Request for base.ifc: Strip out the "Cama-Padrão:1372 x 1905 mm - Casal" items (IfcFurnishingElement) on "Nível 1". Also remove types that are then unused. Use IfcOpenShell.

First a look at what the model holds.

```python
import ifcopenshell
import ifcopenshell.util.element

model = ifcopenshell.open("base.ifc")
print(model.schema)
storey = next(s for s in model.by_type("IfcBuildingStorey") if s.Name == "Nível 1")
furniture = [e for e in ifcopenshell.util.element.get_decomposition(storey) if e.is_a("IfcFurnishingElement")]
seen = {}
for e in furniture:
    element_type = ifcopenshell.util.element.get_type(e)
    name = element_type.Name if element_type not in (None, e) else None
    seen[name] = seen.get(name, 0) + 1
for name, count in sorted(seen.items(), key=str):
    print(count, "x", name)
```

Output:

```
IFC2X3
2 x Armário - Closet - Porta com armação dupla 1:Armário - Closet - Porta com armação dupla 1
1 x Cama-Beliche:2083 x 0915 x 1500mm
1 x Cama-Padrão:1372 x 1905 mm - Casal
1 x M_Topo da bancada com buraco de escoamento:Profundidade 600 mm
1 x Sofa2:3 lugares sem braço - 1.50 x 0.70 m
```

```python
import ifcopenshell
import ifcopenshell.api.root
import ifcopenshell.util.element

model = ifcopenshell.open("base.ifc")

storey = next(s for s in model.by_type("IfcBuildingStorey") if s.Name == "Nível 1")
furniture = [e for e in ifcopenshell.util.element.get_decomposition(storey) if e.is_a("IfcFurnishingElement")]
targets = [e for e in furniture if (t := ifcopenshell.util.element.get_type(e)) not in (None, e) and t.Name == "Cama-Padrão:1372 x 1905 mm - Casal"]
types = {ifcopenshell.util.element.get_type(e) for e in targets} - {None, *targets}

for e in targets:
    ifcopenshell.api.root.remove_product(model, product=e)
print(len(targets), "removed")

unused = [t for t in types if not ifcopenshell.util.element.get_types(t)]
for t in unused:
    ifcopenshell.api.root.remove_product(model, product=t)
print(len(unused), "unused types removed")

model.write("base-out.ifc")
```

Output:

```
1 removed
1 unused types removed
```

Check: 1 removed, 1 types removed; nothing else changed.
